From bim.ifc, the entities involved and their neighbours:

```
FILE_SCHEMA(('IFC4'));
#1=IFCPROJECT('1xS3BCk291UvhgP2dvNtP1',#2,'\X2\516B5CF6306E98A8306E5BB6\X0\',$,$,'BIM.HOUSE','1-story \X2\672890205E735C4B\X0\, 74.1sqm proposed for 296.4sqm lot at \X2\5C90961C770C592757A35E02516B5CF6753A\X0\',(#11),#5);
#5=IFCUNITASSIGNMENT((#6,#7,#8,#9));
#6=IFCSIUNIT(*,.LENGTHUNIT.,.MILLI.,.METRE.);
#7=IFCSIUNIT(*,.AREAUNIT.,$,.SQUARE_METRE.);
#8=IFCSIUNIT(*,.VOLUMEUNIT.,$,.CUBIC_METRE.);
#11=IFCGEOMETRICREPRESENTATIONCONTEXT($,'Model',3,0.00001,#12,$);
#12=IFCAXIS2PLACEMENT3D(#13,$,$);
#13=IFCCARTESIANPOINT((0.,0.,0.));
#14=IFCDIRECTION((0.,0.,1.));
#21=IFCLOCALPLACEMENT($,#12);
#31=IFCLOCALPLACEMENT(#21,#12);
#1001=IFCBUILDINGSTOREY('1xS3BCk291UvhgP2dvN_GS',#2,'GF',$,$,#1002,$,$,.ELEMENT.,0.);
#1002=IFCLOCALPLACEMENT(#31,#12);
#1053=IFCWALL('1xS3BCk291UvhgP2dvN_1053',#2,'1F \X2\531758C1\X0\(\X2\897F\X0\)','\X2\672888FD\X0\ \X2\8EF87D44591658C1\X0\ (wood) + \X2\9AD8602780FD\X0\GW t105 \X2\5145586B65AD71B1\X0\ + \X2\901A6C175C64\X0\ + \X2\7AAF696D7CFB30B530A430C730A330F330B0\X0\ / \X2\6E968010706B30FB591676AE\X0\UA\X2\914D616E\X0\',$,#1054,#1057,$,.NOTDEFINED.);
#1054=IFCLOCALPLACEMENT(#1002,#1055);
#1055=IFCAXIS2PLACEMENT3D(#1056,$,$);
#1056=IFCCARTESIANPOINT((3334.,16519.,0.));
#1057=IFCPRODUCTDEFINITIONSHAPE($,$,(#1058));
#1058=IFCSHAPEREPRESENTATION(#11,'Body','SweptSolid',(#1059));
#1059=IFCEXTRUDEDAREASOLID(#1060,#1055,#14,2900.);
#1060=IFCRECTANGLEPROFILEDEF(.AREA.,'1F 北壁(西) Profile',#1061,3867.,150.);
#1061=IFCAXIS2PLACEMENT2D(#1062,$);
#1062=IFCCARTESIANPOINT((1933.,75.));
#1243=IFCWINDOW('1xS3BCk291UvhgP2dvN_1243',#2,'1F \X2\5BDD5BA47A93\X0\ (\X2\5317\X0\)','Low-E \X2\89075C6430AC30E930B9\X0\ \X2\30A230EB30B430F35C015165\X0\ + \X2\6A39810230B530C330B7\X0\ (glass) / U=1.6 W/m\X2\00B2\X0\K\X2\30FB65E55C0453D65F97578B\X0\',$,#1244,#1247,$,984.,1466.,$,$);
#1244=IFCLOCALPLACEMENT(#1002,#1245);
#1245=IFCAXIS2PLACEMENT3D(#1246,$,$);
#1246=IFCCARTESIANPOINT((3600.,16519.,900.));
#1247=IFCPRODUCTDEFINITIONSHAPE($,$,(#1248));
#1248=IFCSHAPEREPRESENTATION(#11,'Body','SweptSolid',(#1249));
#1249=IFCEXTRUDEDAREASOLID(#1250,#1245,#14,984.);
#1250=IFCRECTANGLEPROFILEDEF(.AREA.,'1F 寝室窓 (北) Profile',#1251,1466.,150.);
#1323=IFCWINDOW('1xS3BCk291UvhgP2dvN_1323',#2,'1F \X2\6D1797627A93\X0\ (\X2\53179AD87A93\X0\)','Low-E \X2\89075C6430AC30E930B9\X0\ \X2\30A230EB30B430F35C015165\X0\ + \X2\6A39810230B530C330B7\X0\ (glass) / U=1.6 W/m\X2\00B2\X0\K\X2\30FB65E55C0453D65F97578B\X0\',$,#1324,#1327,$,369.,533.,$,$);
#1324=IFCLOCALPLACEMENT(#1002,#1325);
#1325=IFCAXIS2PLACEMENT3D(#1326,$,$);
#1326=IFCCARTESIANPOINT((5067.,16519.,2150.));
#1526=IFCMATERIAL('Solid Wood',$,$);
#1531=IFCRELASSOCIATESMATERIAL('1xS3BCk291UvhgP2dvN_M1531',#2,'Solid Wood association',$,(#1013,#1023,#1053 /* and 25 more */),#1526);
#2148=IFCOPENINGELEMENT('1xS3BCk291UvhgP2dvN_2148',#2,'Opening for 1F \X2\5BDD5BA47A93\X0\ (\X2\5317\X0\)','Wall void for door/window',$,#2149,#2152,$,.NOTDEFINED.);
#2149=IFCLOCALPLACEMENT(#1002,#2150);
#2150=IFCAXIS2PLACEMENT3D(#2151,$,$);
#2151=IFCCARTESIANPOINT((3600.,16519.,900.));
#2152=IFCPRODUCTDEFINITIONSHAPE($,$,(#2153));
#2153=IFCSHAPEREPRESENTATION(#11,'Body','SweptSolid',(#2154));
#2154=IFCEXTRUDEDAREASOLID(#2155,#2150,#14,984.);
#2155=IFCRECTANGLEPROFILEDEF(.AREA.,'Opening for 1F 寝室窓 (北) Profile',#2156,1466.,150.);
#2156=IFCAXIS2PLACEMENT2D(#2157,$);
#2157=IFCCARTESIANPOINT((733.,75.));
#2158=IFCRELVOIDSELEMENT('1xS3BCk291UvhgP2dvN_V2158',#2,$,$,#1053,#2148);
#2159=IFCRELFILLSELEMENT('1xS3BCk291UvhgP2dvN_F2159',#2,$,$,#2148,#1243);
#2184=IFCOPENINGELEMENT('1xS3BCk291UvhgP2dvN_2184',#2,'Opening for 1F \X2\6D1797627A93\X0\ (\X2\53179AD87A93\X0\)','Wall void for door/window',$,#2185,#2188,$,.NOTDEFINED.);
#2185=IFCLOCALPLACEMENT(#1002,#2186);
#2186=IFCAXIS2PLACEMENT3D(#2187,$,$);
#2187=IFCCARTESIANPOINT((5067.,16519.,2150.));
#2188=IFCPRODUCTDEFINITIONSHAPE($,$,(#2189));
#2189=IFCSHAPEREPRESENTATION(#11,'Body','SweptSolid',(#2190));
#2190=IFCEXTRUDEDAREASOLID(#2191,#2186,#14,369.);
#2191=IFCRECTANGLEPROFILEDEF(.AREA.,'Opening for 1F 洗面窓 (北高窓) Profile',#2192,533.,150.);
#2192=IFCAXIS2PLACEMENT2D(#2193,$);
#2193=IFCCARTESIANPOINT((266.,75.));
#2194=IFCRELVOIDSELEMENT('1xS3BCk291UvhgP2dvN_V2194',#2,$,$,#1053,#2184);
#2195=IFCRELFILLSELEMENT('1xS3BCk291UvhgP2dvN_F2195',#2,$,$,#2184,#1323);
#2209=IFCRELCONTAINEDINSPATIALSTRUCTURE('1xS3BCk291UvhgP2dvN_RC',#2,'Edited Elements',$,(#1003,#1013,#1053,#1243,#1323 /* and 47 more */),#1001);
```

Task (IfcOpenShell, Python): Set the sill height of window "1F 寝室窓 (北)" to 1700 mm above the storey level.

```python
import numpy as np
import ifcopenshell
import ifcopenshell.api.geometry
import ifcopenshell.geom
import ifcopenshell.util.element
import ifcopenshell.util.placement
import ifcopenshell.util.shape
import ifcopenshell.util.unit

model = ifcopenshell.open("bim.ifc")
unit_scale = ifcopenshell.util.unit.calculate_unit_scale(model)

window = model.by_guid("1xS3BCk291UvhgP2dvN_1243")
opening = window.FillsVoids[0].RelatingOpeningElement
storey = ifcopenshell.util.element.get_container(window, ifc_class="IfcBuildingStorey")
level = ifcopenshell.util.placement.get_local_placement(storey.ObjectPlacement)[2, 3]

# The opening's origin need not be at the sill, so measure its lowest point.
shape = ifcopenshell.geom.create_shape(ifcopenshell.geom.settings(), opening)
bottom = ifcopenshell.util.shape.get_shape_bottom_elevation(shape, shape.geometry) / unit_scale
dz = level + 1700.0 - bottom

shift = np.array([0.0, 0.0, dz])
# The window is not placed relative to its opening, so move both.
for product in (opening, window):
    matrix = ifcopenshell.util.placement.get_local_placement(product.ObjectPlacement)
    matrix[:3, 3] += shift
    ifcopenshell.api.geometry.edit_object_placement(model, product=product, matrix=matrix, is_si=False)

print(f"moved by {dz * unit_scale:+.3f} m")

model.write("bim_v2.ifc")
```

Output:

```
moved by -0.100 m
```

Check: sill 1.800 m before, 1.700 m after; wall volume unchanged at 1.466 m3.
